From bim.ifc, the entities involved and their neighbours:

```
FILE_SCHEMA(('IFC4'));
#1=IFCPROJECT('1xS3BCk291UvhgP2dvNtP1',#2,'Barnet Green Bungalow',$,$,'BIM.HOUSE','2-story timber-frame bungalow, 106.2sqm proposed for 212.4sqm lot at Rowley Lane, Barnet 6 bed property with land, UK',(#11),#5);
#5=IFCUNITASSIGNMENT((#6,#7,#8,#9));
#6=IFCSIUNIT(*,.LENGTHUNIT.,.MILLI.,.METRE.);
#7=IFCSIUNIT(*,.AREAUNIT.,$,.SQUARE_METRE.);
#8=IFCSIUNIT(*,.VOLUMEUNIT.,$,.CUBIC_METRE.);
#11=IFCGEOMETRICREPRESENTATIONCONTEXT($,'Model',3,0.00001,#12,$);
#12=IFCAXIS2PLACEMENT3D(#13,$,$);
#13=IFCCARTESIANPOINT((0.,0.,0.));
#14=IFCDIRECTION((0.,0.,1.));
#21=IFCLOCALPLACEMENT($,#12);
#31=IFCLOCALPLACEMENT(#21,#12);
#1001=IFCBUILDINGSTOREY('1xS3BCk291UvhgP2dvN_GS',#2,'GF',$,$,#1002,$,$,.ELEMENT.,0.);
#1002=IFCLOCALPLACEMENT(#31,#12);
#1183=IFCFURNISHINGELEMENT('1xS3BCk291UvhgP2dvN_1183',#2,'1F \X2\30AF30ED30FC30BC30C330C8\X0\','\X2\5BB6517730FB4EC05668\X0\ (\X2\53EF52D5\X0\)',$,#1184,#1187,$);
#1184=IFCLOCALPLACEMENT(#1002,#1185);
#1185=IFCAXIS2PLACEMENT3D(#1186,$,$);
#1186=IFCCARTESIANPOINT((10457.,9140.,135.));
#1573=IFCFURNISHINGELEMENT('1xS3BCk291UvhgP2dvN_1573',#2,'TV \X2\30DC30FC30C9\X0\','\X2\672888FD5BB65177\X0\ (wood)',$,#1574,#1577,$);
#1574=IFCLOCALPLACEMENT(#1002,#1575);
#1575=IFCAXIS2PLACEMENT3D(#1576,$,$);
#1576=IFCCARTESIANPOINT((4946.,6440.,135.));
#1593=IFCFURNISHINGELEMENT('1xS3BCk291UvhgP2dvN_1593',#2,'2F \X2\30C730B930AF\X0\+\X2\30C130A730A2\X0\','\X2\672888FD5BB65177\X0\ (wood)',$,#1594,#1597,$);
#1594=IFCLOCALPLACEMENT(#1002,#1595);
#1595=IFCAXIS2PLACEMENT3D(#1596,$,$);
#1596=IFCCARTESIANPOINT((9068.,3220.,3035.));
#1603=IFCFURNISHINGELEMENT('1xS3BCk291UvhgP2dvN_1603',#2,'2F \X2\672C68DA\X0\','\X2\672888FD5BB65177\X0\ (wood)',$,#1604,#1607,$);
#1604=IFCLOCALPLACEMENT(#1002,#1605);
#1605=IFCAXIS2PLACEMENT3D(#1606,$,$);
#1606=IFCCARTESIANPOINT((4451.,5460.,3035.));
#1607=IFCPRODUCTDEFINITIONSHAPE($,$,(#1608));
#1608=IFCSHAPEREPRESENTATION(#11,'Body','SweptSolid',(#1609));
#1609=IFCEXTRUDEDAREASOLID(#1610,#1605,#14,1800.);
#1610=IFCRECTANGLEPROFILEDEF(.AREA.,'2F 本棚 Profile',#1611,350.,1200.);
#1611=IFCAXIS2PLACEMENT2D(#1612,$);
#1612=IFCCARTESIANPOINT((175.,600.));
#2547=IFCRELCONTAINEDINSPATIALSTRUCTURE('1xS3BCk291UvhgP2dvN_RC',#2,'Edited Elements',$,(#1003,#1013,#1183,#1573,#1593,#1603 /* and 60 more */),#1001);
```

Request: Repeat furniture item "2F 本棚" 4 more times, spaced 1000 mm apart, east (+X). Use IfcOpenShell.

```python
import numpy as np
import ifcopenshell
import ifcopenshell.api.geometry
import ifcopenshell.api.root
import ifcopenshell.util.element
import ifcopenshell.util.placement

model = ifcopenshell.open("bim.ifc")


def reuse_history(source, copy):
    """copy_class also copies each property set's owner history, people and application; keep the originals."""
    for rel in copy.IsDefinedBy:
        if rel.is_a("IfcRelDefinesByProperties") and (history := rel.RelatingPropertyDefinition.OwnerHistory):
            rel.RelatingPropertyDefinition.OwnerHistory = source.OwnerHistory
            ifcopenshell.util.element.remove_deep2(model, history)


source = model.by_guid("1xS3BCk291UvhgP2dvN_1603")
base = ifcopenshell.util.placement.get_local_placement(source.ObjectPlacement)
step = np.array([1.0, 0.0, 0.0]) * 1000.0

for i in range(1, 5):
    copy = ifcopenshell.api.root.copy_class(model, product=source)
    copy.Representation = ifcopenshell.util.element.copy_deep(
        model, source.Representation, exclude=["IfcGeometricRepresentationContext", "IfcRepresentationMap"]
    )
    reuse_history(source, copy)
    matrix = base.copy()
    matrix[:3, 3] += i * step
    print("added at", matrix[:3, 3].round(3) + 0.0)
    ifcopenshell.api.geometry.edit_object_placement(model, product=copy, matrix=matrix, is_si=False)

model.write("bim-out.ifc")
```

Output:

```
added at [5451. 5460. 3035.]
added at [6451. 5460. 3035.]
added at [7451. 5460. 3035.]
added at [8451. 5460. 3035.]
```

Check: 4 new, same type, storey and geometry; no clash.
